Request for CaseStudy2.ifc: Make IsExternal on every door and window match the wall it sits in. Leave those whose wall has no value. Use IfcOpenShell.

First a look at what the model holds.

```python
import ifcopenshell
import ifcopenshell.util.element

model = ifcopenshell.open("CaseStudy2.ifc")
print(model.schema)
seen = {}
for e in model.by_type("IfcDoor") + model.by_type("IfcWindow"):
    if not e.FillsVoids:
        continue
    host = e.FillsVoids[0].RelatingOpeningElement.VoidsElements[0].RelatingBuildingElement
    own = ifcopenshell.util.element.get_pset(e, f"Pset_{e.is_a()[3:].removesuffix('StandardCase')}Common", "IsExternal")
    wall = ifcopenshell.util.element.get_pset(host, "Pset_WallCommon", "IsExternal")
    seen[e.is_a(), own, wall] = seen.get((e.is_a(), own, wall), 0) + 1
for (cls, own, wall), count in sorted(seen.items(), key=str):
    print(count, cls, "IsExternal:", own, "| host wall:", wall)
```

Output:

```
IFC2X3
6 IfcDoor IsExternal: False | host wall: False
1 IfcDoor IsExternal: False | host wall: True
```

```python
import ifcopenshell
import ifcopenshell.api.pset
import ifcopenshell.util.element

model = ifcopenshell.open("CaseStudy2.ifc")

count = 0
for ifc_class, pset_name in (("IfcDoor", "Pset_DoorCommon"), ("IfcWindow", "Pset_WindowCommon")):
    for e in model.by_type(ifc_class):
        if not e.FillsVoids:
            continue
        host = e.FillsVoids[0].RelatingOpeningElement.VoidsElements[0].RelatingBuildingElement
        external = ifcopenshell.util.element.get_pset(host, "Pset_WallCommon", "IsExternal")
        if external is None or ifcopenshell.util.element.get_pset(e, pset_name, "IsExternal") == external:
            continue
        pset = ifcopenshell.api.pset.add_pset(model, product=e, name=pset_name)
        ifcopenshell.api.pset.edit_pset(model, pset=pset, properties={"IsExternal": external})
        count += 1

print(count, "updated")

model.write("CaseStudy2_rev.ifc")
```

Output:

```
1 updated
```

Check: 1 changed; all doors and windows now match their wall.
